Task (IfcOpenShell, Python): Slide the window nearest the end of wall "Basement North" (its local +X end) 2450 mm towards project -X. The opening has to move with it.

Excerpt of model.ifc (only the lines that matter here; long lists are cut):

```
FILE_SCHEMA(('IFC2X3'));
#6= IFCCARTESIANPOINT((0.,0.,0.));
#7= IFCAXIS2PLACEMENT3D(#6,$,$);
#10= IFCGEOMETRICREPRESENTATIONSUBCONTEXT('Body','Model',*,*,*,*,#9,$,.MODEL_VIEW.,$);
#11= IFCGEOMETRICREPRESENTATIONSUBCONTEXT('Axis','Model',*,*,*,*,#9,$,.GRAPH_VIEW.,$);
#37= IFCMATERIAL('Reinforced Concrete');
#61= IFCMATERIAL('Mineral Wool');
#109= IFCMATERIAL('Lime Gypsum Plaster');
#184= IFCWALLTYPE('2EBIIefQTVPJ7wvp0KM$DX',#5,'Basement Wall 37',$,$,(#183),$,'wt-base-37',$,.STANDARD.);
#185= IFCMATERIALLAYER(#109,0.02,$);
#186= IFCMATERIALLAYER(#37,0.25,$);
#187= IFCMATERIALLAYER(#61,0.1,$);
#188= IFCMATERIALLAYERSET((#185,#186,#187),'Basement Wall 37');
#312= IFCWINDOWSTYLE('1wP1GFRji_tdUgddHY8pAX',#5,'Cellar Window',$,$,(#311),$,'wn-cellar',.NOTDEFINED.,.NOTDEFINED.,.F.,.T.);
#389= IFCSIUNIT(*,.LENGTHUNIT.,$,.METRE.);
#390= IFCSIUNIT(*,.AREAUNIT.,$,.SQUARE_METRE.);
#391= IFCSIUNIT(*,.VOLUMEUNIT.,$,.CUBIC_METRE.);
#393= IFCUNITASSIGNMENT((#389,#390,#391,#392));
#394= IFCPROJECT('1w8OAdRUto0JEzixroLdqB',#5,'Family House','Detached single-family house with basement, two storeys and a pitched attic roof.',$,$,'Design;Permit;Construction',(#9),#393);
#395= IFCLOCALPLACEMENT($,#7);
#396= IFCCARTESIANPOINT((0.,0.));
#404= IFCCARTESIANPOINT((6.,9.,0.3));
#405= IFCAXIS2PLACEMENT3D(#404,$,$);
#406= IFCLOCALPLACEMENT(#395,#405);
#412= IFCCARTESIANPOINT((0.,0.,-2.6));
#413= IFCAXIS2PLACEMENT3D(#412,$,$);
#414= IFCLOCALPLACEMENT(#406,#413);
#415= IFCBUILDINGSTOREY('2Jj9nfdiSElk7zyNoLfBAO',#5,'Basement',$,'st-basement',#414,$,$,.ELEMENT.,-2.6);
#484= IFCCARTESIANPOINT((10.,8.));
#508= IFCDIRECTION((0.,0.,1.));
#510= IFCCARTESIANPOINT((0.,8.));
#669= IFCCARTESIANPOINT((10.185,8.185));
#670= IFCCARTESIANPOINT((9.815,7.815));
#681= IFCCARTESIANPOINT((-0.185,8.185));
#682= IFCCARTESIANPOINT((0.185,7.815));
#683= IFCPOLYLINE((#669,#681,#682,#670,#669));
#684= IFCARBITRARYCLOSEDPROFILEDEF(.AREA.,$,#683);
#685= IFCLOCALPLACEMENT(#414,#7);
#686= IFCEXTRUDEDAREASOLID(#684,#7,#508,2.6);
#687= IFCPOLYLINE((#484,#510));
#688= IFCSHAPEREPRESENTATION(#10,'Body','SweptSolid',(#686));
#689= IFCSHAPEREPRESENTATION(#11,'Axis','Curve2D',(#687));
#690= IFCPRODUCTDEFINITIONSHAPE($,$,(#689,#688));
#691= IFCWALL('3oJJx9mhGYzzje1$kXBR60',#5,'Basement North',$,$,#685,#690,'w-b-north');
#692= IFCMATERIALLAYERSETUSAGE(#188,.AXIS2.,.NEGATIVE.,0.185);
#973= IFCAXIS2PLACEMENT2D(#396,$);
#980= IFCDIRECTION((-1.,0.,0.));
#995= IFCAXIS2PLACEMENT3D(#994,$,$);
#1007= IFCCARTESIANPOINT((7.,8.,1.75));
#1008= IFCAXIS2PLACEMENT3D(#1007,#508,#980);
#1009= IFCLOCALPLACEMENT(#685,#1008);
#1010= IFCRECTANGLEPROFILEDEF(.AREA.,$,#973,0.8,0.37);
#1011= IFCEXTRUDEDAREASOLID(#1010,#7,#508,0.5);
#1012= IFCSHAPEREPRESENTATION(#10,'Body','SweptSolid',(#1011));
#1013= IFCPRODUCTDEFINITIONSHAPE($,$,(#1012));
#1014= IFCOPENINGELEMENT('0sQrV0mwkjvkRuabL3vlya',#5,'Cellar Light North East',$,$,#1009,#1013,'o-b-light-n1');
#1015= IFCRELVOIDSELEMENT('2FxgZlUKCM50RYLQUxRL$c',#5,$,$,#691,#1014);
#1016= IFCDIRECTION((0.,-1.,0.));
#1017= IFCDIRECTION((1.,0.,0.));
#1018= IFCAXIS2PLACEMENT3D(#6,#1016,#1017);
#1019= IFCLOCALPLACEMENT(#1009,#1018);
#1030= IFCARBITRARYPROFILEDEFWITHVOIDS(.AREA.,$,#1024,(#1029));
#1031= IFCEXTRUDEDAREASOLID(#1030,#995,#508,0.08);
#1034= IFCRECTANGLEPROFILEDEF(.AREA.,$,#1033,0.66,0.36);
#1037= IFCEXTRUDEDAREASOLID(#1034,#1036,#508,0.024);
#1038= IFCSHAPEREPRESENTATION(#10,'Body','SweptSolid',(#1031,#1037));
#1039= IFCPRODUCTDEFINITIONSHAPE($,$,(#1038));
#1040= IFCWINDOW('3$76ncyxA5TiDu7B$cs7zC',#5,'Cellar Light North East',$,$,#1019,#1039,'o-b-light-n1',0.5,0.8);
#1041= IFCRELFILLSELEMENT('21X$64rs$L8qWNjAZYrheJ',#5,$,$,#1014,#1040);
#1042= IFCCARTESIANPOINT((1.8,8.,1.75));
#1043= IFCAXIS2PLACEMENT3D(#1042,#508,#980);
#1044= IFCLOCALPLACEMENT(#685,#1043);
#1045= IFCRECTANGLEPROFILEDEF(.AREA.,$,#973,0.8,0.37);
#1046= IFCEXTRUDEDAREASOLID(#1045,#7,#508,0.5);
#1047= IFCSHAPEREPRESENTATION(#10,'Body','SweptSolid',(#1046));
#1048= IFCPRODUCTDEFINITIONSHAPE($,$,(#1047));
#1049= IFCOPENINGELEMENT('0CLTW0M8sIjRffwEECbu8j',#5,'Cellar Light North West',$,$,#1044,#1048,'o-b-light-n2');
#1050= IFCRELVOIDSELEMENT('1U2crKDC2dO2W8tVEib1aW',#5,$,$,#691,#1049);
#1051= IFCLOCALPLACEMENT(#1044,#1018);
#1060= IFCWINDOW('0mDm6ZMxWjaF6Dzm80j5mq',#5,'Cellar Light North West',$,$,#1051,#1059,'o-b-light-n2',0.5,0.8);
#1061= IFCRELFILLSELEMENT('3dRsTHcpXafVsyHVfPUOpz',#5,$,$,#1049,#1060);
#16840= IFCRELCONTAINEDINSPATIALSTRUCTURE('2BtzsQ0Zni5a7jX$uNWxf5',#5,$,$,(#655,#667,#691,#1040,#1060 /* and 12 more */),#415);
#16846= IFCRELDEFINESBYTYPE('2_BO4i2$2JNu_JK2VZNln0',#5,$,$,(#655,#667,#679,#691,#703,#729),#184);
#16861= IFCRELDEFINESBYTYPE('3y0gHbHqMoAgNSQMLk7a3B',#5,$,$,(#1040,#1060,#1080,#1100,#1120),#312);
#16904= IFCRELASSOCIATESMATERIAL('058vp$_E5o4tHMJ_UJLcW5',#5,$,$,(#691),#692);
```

```python
import ifcopenshell
import ifcopenshell.api.geometry
import ifcopenshell.util.placement
import ifcopenshell.util.unit

model = ifcopenshell.open("model.ifc")
unit_scale = ifcopenshell.util.unit.calculate_unit_scale(model)

window = model.by_guid("3$76ncyxA5TiDu7B$cs7zC")
opening = window.FillsVoids[0].RelatingOpeningElement
wall = opening.VoidsElements[0].RelatingBuildingElement

wall_matrix = ifcopenshell.util.placement.get_local_placement(wall.ObjectPlacement)
shift = wall_matrix[:3, 0] * -2.45 / unit_scale
before = ifcopenshell.util.placement.get_local_placement(window.ObjectPlacement)[:3, 3].copy()

# The window is placed relative to its opening, so it follows when the opening moves.
matrix = ifcopenshell.util.placement.get_local_placement(opening.ObjectPlacement)
matrix[:3, 3] += shift
ifcopenshell.api.geometry.edit_object_placement(
    model, product=opening, matrix=matrix, is_si=False, should_transform_children=True
)

after = ifcopenshell.util.placement.get_local_placement(window.ObjectPlacement)[:3, 3]
print("window moved by", (after - before).round(3) + 0.0)

model.write("model_edited.ifc")
```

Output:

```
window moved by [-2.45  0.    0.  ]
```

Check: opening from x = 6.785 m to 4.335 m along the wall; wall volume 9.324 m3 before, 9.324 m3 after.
